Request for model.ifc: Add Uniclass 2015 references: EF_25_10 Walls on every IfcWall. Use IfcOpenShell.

First a look at what the model holds.

```python
import ifcopenshell

model = ifcopenshell.open("model.ifc")
print(model.schema)
print("classifications:", [c.Name for c in model.by_type("IfcClassification")])
for ifc_class in ("IfcDoor", "IfcRoof", "IfcStair", "IfcWall", "IfcWindow"):
    print(ifc_class, len(model.by_type(ifc_class)))
```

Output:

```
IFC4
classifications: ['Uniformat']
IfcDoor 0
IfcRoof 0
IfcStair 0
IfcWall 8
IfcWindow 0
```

```python
import ifcopenshell
import ifcopenshell.api.classification

model = ifcopenshell.open("model.ifc")

system = ifcopenshell.api.classification.add_classification(model, classification="Uniclass 2015")

codes = {
    "IfcWall": ("EF_25_10", "Walls"),
}
for ifc_class, (code, name) in codes.items():
    products = model.by_type(ifc_class)
    ifcopenshell.api.classification.add_reference(
        model, products=products, classification=system, identification=code, name=name
    )
    print(code, len(products))

model.write("model-out.ifc")
```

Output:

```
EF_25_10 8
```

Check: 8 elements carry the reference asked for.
